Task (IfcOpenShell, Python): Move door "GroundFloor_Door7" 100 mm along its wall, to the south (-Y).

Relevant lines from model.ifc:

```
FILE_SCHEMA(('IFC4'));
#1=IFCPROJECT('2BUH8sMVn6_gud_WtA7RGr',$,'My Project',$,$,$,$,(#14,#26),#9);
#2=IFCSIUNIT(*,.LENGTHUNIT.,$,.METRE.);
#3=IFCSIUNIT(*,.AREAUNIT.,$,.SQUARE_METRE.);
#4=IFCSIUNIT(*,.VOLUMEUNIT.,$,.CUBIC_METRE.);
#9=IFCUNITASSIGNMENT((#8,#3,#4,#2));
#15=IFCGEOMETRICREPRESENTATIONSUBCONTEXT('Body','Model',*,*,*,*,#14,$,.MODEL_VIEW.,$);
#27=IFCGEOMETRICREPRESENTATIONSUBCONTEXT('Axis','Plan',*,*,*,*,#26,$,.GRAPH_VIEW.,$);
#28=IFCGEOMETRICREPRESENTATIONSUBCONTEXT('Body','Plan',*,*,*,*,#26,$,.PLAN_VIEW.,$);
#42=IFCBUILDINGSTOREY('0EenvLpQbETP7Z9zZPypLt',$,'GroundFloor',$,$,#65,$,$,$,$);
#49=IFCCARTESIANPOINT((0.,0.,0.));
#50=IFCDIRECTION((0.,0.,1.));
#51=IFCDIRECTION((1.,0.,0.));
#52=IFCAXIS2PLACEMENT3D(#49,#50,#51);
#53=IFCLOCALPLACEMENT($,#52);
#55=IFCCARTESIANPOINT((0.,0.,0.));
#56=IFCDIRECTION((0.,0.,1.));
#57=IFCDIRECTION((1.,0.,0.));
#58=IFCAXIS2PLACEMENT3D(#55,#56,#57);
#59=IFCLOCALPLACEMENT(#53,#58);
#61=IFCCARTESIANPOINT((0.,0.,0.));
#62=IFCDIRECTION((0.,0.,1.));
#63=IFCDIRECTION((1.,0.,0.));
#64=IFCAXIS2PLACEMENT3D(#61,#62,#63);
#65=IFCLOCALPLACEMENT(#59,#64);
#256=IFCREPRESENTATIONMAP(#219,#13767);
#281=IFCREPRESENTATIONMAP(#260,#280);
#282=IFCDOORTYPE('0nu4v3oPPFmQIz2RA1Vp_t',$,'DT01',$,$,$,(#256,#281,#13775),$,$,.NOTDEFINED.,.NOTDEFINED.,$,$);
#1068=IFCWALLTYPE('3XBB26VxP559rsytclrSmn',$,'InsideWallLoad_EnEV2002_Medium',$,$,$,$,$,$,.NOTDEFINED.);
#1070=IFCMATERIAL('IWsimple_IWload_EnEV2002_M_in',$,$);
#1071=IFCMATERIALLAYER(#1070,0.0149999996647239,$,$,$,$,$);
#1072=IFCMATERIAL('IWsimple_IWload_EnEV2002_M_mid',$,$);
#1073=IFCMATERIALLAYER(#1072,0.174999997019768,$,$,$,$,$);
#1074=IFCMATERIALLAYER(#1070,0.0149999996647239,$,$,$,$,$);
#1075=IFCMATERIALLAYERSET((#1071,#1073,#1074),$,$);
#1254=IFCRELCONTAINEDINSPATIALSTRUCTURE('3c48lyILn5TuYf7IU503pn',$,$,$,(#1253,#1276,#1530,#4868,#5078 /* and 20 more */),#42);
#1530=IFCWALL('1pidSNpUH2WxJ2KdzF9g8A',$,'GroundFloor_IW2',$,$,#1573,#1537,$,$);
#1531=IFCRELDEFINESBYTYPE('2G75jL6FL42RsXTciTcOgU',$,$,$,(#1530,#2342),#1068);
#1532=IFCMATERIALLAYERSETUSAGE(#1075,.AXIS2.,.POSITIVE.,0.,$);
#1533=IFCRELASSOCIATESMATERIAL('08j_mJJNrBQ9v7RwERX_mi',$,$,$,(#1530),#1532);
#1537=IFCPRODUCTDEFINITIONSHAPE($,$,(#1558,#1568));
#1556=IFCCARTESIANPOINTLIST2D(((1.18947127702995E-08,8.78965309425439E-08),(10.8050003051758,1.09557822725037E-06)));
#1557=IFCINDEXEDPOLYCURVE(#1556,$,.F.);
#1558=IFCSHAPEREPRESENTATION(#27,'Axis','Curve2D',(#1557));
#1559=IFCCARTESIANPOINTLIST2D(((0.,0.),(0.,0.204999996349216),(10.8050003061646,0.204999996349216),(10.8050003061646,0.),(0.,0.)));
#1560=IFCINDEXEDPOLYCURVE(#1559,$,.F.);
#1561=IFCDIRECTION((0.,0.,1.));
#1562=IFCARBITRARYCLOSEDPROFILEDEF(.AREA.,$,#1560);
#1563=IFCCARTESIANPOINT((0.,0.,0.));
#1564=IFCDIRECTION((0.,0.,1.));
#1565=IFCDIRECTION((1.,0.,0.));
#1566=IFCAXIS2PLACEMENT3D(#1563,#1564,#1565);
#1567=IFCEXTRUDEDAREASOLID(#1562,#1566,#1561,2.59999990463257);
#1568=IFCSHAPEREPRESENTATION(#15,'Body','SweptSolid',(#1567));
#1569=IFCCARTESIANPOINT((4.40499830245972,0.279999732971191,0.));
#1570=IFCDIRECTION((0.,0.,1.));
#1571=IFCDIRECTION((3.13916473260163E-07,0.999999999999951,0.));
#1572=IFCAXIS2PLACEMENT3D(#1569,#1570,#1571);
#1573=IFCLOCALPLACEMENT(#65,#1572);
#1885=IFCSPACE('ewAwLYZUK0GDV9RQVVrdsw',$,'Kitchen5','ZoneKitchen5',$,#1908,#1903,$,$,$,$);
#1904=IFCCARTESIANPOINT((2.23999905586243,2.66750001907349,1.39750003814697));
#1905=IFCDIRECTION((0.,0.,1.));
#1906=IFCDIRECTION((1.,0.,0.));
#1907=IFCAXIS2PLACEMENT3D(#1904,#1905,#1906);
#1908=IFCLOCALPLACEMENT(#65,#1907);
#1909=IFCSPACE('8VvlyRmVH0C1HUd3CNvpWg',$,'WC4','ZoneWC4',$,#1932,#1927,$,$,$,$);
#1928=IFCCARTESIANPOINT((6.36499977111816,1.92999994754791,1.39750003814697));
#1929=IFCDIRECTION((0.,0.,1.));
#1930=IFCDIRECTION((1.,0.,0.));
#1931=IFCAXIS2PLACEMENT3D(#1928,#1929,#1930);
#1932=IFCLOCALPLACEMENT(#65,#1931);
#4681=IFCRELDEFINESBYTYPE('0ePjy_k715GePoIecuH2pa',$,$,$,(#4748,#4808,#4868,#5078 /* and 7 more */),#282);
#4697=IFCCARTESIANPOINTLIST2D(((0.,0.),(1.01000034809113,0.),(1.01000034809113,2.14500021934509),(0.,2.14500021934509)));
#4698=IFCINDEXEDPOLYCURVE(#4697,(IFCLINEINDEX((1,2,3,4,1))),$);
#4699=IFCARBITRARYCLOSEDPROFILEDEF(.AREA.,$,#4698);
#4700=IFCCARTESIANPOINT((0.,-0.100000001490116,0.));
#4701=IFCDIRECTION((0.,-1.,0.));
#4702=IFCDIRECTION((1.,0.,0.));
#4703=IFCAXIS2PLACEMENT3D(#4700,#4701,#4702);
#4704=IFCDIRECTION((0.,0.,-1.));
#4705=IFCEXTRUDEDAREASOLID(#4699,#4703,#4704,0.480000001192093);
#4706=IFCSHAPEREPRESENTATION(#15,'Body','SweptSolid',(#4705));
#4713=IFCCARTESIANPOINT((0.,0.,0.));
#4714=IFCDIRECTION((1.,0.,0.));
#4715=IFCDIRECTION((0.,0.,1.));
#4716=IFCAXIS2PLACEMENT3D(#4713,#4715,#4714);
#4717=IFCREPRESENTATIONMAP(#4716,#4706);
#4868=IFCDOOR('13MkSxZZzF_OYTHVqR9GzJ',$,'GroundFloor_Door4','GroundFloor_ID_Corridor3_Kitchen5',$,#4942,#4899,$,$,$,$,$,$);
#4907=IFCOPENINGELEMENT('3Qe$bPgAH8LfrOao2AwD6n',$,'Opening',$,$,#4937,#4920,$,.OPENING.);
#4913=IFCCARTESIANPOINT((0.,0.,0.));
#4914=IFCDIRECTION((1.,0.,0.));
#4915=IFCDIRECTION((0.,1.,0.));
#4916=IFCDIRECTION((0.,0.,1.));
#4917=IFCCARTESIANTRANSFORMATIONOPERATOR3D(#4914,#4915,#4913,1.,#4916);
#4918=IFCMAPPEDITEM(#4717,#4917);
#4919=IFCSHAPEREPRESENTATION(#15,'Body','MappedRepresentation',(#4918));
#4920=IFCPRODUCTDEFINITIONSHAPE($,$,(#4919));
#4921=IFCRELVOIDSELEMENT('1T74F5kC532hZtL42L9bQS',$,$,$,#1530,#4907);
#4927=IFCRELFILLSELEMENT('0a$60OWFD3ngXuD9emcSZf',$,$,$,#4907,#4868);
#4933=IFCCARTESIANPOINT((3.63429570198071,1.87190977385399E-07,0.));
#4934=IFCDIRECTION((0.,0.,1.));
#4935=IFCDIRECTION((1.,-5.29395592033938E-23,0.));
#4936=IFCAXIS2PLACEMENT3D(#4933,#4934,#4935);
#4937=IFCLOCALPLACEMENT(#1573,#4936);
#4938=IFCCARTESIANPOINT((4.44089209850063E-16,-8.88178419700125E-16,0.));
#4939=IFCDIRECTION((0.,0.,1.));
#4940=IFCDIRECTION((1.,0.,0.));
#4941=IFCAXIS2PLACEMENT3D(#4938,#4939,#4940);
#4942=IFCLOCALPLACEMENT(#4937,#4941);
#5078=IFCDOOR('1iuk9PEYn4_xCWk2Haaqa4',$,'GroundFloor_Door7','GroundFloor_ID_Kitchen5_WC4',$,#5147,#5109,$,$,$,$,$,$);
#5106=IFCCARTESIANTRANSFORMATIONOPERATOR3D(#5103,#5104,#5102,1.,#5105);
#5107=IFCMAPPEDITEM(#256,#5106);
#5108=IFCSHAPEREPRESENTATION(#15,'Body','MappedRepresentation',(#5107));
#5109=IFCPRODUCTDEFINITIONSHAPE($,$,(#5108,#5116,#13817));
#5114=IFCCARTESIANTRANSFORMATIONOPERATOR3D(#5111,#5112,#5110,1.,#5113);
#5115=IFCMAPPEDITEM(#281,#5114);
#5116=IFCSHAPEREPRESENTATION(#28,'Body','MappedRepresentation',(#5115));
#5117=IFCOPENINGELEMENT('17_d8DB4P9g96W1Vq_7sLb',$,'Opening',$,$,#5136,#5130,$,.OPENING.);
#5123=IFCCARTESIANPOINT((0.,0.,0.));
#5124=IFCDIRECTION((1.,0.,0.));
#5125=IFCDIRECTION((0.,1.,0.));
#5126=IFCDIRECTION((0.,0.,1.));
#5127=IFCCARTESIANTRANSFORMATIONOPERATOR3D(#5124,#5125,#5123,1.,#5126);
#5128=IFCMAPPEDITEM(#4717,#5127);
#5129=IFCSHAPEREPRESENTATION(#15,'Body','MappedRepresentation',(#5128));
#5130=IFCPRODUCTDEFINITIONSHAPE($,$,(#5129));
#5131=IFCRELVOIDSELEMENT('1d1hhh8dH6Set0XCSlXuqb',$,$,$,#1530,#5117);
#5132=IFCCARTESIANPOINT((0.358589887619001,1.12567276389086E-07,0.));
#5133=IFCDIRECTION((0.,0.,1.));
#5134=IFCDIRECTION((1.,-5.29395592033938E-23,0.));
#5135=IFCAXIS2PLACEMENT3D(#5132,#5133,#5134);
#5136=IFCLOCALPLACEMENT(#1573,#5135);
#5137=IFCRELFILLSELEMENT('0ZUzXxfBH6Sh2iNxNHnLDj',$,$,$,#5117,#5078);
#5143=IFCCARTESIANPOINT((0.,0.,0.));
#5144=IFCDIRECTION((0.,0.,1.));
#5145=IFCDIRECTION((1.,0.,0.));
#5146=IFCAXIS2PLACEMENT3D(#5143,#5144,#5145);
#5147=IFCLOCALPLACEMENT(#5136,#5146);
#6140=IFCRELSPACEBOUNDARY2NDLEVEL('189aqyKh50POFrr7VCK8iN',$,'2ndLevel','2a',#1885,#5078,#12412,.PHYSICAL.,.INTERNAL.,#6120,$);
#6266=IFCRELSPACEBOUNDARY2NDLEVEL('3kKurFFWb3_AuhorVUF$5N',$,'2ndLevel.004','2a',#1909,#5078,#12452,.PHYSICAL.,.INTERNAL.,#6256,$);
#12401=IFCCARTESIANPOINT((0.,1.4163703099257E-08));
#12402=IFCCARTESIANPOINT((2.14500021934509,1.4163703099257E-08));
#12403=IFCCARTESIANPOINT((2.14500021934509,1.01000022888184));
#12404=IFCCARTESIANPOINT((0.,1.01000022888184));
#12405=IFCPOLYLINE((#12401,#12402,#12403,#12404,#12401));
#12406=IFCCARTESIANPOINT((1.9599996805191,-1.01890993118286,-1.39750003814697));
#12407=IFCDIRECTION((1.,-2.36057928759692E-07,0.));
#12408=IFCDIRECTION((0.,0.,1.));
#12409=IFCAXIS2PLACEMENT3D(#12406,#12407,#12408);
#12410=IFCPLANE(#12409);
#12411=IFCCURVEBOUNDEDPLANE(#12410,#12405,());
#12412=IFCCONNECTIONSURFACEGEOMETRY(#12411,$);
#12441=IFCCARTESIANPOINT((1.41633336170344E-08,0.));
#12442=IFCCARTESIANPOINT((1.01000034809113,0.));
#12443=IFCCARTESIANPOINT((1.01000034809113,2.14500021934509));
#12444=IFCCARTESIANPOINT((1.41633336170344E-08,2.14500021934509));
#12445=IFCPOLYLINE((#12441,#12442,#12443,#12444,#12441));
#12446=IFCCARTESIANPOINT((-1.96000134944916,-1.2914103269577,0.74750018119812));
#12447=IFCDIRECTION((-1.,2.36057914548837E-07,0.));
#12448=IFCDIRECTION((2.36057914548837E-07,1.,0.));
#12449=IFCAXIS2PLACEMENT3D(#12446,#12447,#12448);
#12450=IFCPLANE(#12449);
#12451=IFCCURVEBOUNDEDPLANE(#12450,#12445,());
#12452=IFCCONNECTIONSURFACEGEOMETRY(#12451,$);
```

```python
import numpy as np
import ifcopenshell
import ifcopenshell.api.geometry
import ifcopenshell.util.placement
import ifcopenshell.util.unit

model = ifcopenshell.open("model.ifc")
unit_scale = ifcopenshell.util.unit.calculate_unit_scale(model)

door = model.by_guid("1iuk9PEYn4_xCWk2Haaqa4")
opening = door.FillsVoids[0].RelatingOpeningElement
wall = opening.VoidsElements[0].RelatingBuildingElement

wall_matrix = ifcopenshell.util.placement.get_local_placement(wall.ObjectPlacement)
shift = wall_matrix[:3, 0] * -0.1 / unit_scale
before = ifcopenshell.util.placement.get_local_placement(door.ObjectPlacement)[:3, 3].copy()

# The door is placed relative to its opening, so it follows when the opening moves.
matrix = ifcopenshell.util.placement.get_local_placement(opening.ObjectPlacement)
matrix[:3, 3] += shift
ifcopenshell.api.geometry.edit_object_placement(
    model, product=opening, matrix=matrix, is_si=False, should_transform_children=True
)

# Space boundary surfaces are stored in each space's coordinates; move them too.
for rel in door.ProvidesBoundaries:
    if not rel.ConnectionGeometry:
        continue
    surface = rel.ConnectionGeometry.SurfaceOnRelatingElement.BasisSurface
    space_matrix = ifcopenshell.util.placement.get_local_placement(rel.RelatingSpace.ObjectPlacement)
    point = np.array(surface.Position.Location.Coordinates) + space_matrix[:3, :3].T @ shift
    surface.Position = model.createIfcAxis2Placement3D(
        model.createIfcCartesianPoint(point.tolist()), surface.Position.Axis, surface.Position.RefDirection
    )

after = ifcopenshell.util.placement.get_local_placement(door.ObjectPlacement)[:3, 3]
print("door moved by", (after - before).round(3) + 0.0)

model.write("model-out.ifc")
```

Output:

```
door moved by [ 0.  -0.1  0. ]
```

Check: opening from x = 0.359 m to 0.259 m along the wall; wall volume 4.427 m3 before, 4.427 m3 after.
